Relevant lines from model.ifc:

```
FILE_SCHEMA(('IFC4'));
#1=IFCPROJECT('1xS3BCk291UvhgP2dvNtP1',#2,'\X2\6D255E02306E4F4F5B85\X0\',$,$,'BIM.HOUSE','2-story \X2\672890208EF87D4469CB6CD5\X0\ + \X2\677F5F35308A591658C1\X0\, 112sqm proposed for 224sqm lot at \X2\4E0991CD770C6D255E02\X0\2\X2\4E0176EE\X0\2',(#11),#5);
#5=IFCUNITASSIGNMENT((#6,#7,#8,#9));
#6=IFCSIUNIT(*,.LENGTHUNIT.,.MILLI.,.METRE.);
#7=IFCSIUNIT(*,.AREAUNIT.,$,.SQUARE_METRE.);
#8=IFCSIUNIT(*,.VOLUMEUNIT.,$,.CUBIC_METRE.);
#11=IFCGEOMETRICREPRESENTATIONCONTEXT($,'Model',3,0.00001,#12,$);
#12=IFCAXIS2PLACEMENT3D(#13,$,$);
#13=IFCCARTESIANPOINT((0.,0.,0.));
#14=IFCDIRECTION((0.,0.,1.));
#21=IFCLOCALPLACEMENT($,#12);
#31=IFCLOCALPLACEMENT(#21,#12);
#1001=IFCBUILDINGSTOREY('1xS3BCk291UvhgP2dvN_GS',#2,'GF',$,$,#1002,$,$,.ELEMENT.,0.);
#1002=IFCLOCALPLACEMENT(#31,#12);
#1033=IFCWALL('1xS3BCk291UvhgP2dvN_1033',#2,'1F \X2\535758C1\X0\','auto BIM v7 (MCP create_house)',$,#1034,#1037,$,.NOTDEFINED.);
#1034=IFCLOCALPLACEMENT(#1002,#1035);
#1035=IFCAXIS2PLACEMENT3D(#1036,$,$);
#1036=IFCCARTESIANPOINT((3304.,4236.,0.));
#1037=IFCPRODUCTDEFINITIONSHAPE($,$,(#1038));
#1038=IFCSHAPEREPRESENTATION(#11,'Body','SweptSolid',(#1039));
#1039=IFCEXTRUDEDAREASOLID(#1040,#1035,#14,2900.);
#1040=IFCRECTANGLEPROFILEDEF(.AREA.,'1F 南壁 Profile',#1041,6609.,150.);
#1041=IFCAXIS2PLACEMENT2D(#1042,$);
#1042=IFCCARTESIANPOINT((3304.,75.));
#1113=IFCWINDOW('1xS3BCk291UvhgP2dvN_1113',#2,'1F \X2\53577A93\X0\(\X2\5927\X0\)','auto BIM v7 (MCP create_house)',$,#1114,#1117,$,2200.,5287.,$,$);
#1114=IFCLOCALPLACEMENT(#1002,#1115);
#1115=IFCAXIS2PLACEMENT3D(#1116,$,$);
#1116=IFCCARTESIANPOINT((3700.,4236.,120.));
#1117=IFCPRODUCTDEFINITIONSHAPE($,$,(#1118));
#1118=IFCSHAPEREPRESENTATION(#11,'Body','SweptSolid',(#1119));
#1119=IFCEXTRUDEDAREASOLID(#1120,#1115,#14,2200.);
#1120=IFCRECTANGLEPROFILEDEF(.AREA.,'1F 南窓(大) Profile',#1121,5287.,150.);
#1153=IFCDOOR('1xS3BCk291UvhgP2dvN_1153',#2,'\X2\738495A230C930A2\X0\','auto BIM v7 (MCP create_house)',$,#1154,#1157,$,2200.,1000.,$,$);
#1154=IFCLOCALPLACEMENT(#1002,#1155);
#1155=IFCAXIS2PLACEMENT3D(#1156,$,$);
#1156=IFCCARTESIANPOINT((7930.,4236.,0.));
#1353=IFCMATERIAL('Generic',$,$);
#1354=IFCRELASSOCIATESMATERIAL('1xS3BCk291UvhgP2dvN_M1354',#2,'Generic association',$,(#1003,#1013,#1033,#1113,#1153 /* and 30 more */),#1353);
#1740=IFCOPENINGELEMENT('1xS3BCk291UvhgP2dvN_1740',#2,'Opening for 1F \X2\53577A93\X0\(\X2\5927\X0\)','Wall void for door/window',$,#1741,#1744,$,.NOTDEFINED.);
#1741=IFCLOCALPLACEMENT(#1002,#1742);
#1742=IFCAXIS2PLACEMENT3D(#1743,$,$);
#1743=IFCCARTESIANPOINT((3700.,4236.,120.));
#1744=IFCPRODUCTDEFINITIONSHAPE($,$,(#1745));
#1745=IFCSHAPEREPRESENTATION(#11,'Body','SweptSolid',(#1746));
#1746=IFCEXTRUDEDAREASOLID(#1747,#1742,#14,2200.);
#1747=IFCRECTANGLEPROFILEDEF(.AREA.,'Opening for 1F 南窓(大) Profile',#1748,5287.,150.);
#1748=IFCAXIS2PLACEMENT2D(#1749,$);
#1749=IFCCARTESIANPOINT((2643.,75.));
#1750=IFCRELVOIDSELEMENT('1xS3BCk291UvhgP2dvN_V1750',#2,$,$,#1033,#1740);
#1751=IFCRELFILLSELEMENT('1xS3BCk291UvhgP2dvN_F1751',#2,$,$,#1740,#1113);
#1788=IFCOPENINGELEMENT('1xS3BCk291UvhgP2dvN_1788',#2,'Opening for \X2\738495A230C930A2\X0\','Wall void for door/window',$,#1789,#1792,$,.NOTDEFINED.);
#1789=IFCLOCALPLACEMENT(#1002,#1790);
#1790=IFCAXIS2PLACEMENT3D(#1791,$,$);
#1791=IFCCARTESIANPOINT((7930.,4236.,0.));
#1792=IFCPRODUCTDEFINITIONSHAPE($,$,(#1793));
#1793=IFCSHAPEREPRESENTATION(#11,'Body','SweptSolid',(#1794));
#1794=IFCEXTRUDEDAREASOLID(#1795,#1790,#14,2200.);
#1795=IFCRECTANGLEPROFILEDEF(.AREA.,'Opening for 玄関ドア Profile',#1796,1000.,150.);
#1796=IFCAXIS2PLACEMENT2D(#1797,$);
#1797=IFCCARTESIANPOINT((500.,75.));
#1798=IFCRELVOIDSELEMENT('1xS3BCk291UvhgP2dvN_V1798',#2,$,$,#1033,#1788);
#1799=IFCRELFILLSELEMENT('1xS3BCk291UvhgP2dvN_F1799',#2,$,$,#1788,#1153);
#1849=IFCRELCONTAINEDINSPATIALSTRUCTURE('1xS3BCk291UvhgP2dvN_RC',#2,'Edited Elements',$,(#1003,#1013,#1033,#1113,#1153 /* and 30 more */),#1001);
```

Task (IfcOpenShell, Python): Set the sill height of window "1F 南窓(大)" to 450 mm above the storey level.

```python
import numpy as np
import ifcopenshell
import ifcopenshell.api.geometry
import ifcopenshell.geom
import ifcopenshell.util.element
import ifcopenshell.util.placement
import ifcopenshell.util.shape
import ifcopenshell.util.unit

model = ifcopenshell.open("model.ifc")
unit_scale = ifcopenshell.util.unit.calculate_unit_scale(model)

window = model.by_guid("1xS3BCk291UvhgP2dvN_1113")
opening = window.FillsVoids[0].RelatingOpeningElement
storey = ifcopenshell.util.element.get_container(window, ifc_class="IfcBuildingStorey")
level = ifcopenshell.util.placement.get_local_placement(storey.ObjectPlacement)[2, 3]

# The opening's origin need not be at the sill, so measure its lowest point.
shape = ifcopenshell.geom.create_shape(ifcopenshell.geom.settings(), opening)
bottom = ifcopenshell.util.shape.get_shape_bottom_elevation(shape, shape.geometry) / unit_scale
dz = level + 0.45 / unit_scale - bottom

shift = np.array([0.0, 0.0, dz])
# The window is not placed relative to its opening, so move both.
for product in (opening, window):
    matrix = ifcopenshell.util.placement.get_local_placement(product.ObjectPlacement)
    matrix[:3, 3] += shift
    ifcopenshell.api.geometry.edit_object_placement(model, product=product, matrix=matrix, is_si=False)

print(f"moved by {dz * unit_scale:+.3f} m")

model.write("model-out.ifc")
```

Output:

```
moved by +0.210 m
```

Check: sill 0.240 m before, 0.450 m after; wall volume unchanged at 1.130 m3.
